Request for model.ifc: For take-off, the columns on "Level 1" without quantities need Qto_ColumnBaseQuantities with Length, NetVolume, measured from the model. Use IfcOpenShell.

First a look at what the model holds.

```python
import ifcopenshell
import ifcopenshell.util.element
import ifcopenshell.util.unit

model = ifcopenshell.open("model.ifc")
print(model.schema)
for unit_type in ("LENGTHUNIT", "AREAUNIT", "VOLUMEUNIT"):
    print(unit_type, ifcopenshell.util.unit.calculate_unit_scale(model, unit_type))
storey = next(s for s in model.by_type("IfcBuildingStorey") if s.Name == "Level 1")
columns = [e for e in ifcopenshell.util.element.get_decomposition(storey) if e.is_a("IfcColumn")]
for e in sorted(columns, key=lambda e: e.id()):
    print(e.id(), e.is_a(), e.Name, list(ifcopenshell.util.element.get_psets(e, qtos_only=True)), sep=" | ")
```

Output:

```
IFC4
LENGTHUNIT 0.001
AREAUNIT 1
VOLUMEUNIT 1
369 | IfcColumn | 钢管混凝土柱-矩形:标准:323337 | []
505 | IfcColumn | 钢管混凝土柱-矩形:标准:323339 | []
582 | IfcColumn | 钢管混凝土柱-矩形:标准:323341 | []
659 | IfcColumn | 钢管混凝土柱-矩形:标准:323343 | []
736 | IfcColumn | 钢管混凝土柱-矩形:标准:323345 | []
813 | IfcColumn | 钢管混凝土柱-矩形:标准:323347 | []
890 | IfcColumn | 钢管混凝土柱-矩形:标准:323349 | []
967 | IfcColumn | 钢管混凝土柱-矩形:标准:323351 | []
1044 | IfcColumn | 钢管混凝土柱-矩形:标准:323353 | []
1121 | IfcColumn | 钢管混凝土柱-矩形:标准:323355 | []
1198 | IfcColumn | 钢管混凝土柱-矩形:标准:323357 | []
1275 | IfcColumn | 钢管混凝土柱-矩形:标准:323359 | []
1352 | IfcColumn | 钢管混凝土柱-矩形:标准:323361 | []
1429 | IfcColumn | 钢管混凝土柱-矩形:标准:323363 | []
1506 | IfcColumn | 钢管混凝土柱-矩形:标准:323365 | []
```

```python
import ifcopenshell
import ifcopenshell.api.pset
import ifcopenshell.geom
import ifcopenshell.util.element
import ifcopenshell.util.shape
import ifcopenshell.util.unit

model = ifcopenshell.open("model.ifc")
unit_scale = ifcopenshell.util.unit.calculate_unit_scale(model)
volume_scale = ifcopenshell.util.unit.calculate_unit_scale(model, "VOLUMEUNIT")
settings = ifcopenshell.geom.settings()

storey = next(s for s in model.by_type("IfcBuildingStorey") if s.Name == "Level 1")
columns = [e for e in ifcopenshell.util.element.get_decomposition(storey) if e.is_a("IfcColumn")]

for e in sorted(columns, key=lambda e: e.id()):
    if ifcopenshell.util.element.get_psets(e, qtos_only=True, should_inherit=False):
        continue
    # Geometry comes back in metres, in the element's own axes.
    shape = ifcopenshell.geom.create_shape(settings, e)
    values = {
        "Length": ifcopenshell.util.shape.get_z(shape.geometry) / unit_scale,
        "NetVolume": ifcopenshell.util.shape.get_volume(shape.geometry) / volume_scale,
    }
    qto = ifcopenshell.api.pset.add_qto(model, product=e, name="Qto_ColumnBaseQuantities")
    ifcopenshell.api.pset.edit_qto(model, qto=qto, properties=values)
    print(e.id(), {k: round(v, 3) for k, v in values.items()})

model.write("model_rev.ifc")
```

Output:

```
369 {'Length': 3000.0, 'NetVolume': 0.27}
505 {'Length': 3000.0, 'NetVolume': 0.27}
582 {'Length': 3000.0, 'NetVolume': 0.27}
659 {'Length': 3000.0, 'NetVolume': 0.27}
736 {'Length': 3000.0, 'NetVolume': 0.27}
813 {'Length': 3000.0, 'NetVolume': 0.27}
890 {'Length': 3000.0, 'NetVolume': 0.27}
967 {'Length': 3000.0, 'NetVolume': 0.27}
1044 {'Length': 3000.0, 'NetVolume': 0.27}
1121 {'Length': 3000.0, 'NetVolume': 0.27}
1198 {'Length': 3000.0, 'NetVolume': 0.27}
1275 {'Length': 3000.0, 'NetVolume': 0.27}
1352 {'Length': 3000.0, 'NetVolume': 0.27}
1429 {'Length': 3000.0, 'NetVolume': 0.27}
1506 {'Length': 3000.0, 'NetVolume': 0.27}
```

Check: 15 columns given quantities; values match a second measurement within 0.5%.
